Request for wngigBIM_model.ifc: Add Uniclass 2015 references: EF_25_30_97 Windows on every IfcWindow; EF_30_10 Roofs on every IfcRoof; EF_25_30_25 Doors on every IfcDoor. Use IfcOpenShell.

First a look at what the model holds.

```python
import ifcopenshell

model = ifcopenshell.open("wngigBIM_model.ifc")
print(model.schema)
print("classifications:", [c.Name for c in model.by_type("IfcClassification")])
for ifc_class in ("IfcDoor", "IfcRoof", "IfcStair", "IfcWall", "IfcWindow"):
    print(ifc_class, len(model.by_type(ifc_class)))
```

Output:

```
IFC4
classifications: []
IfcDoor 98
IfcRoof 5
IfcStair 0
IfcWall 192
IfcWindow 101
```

```python
import ifcopenshell
import ifcopenshell.api.classification

model = ifcopenshell.open("wngigBIM_model.ifc")

system = ifcopenshell.api.classification.add_classification(model, classification="Uniclass 2015")

codes = {
    "IfcWindow": ("EF_25_30_97", "Windows"),
    "IfcRoof": ("EF_30_10", "Roofs"),
    "IfcDoor": ("EF_25_30_25", "Doors"),
}
for ifc_class, (code, name) in codes.items():
    products = model.by_type(ifc_class)
    ifcopenshell.api.classification.add_reference(
        model, products=products, classification=system, identification=code, name=name
    )
    print(code, len(products))

model.write("wngigBIM_model_updated.ifc")
```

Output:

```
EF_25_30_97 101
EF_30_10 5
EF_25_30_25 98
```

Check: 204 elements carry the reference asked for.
